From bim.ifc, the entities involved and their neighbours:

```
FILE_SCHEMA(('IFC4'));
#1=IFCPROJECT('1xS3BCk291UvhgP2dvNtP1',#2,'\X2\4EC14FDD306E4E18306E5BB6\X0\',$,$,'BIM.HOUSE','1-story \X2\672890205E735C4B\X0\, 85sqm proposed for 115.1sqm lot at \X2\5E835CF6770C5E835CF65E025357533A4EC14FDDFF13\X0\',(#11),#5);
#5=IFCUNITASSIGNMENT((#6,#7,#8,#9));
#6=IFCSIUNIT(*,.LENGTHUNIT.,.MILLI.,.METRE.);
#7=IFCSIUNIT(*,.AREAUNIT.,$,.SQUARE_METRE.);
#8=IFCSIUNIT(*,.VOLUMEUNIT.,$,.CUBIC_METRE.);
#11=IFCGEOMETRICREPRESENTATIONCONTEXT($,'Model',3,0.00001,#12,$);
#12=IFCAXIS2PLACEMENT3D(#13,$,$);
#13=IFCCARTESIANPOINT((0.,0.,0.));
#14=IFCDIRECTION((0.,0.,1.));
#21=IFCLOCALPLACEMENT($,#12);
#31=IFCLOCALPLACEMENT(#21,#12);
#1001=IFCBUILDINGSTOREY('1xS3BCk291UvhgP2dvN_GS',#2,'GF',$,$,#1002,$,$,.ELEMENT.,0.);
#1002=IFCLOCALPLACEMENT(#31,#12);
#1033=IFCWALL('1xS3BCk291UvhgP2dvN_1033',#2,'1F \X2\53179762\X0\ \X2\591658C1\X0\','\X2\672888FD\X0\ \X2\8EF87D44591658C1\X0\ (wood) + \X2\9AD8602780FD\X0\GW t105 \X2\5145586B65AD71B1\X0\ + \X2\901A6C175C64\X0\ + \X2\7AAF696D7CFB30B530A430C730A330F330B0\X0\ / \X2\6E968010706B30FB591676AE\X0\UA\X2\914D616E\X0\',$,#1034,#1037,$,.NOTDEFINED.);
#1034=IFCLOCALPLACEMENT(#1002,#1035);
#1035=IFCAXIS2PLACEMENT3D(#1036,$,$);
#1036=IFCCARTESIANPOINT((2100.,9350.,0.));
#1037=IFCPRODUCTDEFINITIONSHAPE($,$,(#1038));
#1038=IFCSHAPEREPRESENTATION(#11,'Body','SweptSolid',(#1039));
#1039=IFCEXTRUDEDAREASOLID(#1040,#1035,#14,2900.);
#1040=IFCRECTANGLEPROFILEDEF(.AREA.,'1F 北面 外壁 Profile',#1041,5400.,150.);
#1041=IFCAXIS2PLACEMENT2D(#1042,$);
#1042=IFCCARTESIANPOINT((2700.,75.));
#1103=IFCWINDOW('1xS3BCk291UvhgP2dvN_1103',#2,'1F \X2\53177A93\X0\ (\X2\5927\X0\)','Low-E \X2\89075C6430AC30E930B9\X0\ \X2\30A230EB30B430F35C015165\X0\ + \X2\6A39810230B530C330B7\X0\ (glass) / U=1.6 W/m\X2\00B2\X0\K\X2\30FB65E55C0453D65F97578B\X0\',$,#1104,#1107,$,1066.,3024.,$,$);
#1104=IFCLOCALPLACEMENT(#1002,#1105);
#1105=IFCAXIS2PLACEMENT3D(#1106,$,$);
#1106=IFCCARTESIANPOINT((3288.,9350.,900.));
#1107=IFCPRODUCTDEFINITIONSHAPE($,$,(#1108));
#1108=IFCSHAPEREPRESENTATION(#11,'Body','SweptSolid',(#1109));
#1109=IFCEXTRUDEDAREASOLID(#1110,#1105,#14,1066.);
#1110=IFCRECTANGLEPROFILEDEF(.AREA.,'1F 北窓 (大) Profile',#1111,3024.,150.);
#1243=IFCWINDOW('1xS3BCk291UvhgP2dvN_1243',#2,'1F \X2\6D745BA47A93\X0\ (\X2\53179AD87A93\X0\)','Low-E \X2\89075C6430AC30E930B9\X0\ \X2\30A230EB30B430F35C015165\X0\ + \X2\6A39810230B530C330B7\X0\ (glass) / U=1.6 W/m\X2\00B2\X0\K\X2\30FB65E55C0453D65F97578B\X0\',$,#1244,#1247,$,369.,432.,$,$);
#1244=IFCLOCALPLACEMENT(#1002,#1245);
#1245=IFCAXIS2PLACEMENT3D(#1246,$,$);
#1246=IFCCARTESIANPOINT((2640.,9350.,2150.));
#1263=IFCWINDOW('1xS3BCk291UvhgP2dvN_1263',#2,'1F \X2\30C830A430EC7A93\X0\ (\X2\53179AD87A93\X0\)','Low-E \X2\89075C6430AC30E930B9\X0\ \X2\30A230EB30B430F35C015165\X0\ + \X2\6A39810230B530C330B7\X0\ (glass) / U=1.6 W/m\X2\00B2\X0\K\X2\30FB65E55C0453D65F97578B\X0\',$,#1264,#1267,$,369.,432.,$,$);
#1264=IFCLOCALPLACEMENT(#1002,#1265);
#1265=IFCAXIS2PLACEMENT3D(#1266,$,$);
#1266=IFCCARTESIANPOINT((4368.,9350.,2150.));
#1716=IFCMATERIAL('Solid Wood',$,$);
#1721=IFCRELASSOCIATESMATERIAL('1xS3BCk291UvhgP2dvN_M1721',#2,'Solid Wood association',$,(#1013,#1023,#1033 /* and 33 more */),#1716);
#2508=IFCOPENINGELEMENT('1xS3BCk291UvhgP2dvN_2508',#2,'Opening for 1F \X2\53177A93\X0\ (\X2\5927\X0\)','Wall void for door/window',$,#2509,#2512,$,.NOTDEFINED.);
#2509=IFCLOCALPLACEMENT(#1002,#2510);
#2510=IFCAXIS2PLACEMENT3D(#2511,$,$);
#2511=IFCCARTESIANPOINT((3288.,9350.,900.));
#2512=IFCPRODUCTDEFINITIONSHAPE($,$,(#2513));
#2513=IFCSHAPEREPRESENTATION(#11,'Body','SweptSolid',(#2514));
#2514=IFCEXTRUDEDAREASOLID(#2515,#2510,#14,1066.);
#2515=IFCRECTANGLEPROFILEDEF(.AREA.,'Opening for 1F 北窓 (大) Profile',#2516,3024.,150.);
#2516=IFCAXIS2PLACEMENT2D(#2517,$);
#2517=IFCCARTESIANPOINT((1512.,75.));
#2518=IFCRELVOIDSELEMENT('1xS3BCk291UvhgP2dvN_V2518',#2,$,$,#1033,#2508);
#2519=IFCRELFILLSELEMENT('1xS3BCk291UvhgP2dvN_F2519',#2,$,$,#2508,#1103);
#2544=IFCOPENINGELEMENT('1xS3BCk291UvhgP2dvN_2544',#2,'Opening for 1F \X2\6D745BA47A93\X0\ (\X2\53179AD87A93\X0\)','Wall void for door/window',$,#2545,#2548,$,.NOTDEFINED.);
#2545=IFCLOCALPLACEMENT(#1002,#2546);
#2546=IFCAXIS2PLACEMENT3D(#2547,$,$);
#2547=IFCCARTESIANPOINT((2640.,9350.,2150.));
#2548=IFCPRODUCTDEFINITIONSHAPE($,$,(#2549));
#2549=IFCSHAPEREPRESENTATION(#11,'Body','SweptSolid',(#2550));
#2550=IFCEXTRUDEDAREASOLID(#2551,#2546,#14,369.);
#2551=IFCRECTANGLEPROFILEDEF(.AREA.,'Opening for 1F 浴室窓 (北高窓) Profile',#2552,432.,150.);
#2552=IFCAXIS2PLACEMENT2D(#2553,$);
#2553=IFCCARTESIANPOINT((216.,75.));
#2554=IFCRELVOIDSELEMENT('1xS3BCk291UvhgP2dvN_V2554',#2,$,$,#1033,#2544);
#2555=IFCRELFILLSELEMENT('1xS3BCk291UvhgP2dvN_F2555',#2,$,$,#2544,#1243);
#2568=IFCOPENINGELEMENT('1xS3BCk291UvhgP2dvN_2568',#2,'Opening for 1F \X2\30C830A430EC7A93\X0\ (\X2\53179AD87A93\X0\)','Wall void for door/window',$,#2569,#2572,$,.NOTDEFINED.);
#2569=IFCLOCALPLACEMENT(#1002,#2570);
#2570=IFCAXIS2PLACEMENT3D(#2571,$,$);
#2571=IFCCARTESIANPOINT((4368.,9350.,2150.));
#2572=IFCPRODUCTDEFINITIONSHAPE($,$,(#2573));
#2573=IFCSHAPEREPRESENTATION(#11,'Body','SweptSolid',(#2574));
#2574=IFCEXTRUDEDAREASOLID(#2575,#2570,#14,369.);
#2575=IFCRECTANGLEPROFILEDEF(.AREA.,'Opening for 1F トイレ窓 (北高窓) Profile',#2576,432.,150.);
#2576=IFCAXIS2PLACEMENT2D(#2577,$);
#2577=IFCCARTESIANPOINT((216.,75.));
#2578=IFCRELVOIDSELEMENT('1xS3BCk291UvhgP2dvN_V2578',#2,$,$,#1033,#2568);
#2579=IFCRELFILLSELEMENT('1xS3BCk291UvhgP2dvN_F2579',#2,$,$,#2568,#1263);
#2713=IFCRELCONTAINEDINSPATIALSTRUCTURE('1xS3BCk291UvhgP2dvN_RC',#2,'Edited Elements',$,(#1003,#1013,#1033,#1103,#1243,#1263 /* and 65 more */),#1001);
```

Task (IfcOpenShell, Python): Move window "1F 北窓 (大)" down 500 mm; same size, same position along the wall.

```python
import numpy as np
import ifcopenshell
import ifcopenshell.api.geometry
import ifcopenshell.util.placement
import ifcopenshell.util.unit

model = ifcopenshell.open("bim.ifc")
unit_scale = ifcopenshell.util.unit.calculate_unit_scale(model)

window = model.by_id(1103)
opening = window.FillsVoids[0].RelatingOpeningElement
dz = -0.5 / unit_scale

shift = np.array([0.0, 0.0, dz])
# The window is not placed relative to its opening, so move both.
for product in (opening, window):
    matrix = ifcopenshell.util.placement.get_local_placement(product.ObjectPlacement)
    matrix[:3, 3] += shift
    ifcopenshell.api.geometry.edit_object_placement(model, product=product, matrix=matrix, is_si=False)

print(f"moved by {dz * unit_scale:+.3f} m")

model.write("bim_v2.ifc")
```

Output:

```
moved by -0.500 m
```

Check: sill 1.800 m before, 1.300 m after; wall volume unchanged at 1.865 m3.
